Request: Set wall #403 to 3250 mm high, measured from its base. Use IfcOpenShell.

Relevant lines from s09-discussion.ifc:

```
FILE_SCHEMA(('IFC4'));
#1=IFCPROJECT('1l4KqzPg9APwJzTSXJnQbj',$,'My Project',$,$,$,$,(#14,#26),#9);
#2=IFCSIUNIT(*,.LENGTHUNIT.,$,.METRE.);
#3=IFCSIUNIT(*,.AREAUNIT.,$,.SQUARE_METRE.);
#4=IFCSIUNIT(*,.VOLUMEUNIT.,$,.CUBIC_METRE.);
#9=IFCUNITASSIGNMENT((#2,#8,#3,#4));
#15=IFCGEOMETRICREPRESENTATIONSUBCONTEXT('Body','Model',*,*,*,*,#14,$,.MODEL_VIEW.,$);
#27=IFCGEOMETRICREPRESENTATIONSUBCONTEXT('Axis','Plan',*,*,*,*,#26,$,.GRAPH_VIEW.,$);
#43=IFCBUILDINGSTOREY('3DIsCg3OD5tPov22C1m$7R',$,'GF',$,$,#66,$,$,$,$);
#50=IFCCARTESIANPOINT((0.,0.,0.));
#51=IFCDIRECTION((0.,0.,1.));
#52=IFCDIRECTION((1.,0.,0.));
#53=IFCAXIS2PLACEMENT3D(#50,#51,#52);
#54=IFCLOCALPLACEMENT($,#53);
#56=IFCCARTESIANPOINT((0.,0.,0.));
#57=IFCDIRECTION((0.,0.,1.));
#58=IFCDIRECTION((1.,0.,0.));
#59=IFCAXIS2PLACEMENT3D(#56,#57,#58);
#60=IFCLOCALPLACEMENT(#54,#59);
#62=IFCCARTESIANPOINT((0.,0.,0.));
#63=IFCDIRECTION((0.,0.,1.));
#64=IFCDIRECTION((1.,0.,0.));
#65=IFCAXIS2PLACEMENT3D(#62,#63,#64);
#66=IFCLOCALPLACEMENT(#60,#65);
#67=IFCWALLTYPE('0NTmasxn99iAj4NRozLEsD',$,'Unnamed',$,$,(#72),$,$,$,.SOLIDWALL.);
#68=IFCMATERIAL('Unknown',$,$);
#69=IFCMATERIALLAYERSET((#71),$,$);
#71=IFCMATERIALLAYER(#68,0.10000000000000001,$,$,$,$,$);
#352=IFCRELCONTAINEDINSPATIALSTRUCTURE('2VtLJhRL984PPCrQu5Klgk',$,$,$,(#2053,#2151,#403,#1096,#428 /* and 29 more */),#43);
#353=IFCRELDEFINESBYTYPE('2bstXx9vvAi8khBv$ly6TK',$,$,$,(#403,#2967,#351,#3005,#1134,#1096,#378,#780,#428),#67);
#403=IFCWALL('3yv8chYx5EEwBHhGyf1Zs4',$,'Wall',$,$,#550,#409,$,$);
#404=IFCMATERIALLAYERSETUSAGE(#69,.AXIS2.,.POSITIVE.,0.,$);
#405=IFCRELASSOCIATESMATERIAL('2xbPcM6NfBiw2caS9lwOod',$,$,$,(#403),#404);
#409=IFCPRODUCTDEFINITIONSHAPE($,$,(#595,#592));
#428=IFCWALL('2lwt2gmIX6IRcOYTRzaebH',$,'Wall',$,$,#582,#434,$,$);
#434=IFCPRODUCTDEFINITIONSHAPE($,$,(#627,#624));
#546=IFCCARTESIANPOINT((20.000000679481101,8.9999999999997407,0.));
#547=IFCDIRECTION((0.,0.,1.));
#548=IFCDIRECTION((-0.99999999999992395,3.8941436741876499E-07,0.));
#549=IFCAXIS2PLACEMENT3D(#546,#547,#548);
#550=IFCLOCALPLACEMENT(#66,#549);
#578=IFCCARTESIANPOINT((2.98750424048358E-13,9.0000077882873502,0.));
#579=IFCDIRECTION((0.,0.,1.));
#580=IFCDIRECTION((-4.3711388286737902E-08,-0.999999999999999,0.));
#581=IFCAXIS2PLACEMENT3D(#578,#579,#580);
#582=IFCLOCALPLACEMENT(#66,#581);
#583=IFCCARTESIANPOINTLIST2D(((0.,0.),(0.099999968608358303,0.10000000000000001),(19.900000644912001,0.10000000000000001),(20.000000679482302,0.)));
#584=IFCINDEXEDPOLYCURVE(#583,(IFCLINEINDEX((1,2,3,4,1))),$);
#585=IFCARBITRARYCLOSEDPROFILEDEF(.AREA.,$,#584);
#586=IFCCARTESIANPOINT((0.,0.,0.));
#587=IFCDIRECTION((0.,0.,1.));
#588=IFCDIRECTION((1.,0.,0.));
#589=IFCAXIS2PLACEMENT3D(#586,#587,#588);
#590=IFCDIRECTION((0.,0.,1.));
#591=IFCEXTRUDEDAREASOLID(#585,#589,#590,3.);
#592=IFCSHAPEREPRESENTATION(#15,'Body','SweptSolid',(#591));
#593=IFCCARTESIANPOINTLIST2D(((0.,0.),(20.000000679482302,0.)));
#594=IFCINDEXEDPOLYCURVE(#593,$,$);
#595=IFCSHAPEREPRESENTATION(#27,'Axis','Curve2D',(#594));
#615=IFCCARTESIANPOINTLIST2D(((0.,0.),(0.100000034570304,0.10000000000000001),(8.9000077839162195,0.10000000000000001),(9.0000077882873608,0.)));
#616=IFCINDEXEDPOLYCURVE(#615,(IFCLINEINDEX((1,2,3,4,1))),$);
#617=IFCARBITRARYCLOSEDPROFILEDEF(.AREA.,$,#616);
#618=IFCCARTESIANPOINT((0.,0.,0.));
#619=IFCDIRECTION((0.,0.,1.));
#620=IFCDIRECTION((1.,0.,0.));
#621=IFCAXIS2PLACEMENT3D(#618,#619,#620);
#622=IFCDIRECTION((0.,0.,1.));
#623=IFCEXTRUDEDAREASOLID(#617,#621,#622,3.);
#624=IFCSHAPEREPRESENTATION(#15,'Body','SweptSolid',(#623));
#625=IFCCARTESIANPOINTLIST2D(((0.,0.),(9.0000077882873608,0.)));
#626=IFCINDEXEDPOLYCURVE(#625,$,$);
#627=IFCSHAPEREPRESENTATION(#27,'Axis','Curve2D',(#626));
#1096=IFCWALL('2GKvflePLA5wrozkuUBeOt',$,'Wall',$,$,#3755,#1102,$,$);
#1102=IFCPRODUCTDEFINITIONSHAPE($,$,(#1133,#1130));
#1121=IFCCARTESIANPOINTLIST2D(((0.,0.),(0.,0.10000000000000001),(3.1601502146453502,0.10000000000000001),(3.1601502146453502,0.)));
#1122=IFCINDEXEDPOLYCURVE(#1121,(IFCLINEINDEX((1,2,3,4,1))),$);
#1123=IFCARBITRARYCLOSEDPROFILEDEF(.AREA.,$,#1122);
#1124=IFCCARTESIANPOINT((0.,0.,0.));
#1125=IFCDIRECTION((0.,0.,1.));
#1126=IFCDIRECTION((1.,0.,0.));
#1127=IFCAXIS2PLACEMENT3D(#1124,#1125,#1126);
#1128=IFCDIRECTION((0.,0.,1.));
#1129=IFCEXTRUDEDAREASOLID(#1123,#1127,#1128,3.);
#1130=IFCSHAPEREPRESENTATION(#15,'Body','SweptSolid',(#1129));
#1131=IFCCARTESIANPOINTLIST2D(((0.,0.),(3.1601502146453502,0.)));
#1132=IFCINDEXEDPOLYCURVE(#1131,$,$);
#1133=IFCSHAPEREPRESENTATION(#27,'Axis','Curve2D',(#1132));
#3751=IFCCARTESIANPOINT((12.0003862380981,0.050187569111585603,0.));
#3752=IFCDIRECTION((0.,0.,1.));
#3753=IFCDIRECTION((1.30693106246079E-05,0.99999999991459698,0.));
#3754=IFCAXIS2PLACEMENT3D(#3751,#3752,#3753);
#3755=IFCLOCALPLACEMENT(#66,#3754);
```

```python
import ifcopenshell
import ifcopenshell.geom
import ifcopenshell.util.representation
import ifcopenshell.util.shape
import ifcopenshell.util.unit

model = ifcopenshell.open("s09-discussion.ifc")
unit_scale = ifcopenshell.util.unit.calculate_unit_scale(model)
settings = ifcopenshell.geom.settings()


def volume(element):
    """Net volume in cubic metres, openings subtracted."""
    shape = ifcopenshell.geom.create_shape(settings, element)
    return ifcopenshell.util.shape.get_volume(shape.geometry)


wall = model.by_guid("3yv8chYx5EEwBHhGyf1Zs4")
before = volume(wall)

body = ifcopenshell.util.representation.get_representation(wall, "Model", "Body")
solid = body.Items[0]
old_height = solid.Depth
solid.Depth = 3.25 / unit_scale
after = volume(wall)

print(f"height {old_height:g} -> {solid.Depth:g}, volume {before:.3f} -> {after:.3f} m3")

model.write("s09-discussion_edited.ifc")
```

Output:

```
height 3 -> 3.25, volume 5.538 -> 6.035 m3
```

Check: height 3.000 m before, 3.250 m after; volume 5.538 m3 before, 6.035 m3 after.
